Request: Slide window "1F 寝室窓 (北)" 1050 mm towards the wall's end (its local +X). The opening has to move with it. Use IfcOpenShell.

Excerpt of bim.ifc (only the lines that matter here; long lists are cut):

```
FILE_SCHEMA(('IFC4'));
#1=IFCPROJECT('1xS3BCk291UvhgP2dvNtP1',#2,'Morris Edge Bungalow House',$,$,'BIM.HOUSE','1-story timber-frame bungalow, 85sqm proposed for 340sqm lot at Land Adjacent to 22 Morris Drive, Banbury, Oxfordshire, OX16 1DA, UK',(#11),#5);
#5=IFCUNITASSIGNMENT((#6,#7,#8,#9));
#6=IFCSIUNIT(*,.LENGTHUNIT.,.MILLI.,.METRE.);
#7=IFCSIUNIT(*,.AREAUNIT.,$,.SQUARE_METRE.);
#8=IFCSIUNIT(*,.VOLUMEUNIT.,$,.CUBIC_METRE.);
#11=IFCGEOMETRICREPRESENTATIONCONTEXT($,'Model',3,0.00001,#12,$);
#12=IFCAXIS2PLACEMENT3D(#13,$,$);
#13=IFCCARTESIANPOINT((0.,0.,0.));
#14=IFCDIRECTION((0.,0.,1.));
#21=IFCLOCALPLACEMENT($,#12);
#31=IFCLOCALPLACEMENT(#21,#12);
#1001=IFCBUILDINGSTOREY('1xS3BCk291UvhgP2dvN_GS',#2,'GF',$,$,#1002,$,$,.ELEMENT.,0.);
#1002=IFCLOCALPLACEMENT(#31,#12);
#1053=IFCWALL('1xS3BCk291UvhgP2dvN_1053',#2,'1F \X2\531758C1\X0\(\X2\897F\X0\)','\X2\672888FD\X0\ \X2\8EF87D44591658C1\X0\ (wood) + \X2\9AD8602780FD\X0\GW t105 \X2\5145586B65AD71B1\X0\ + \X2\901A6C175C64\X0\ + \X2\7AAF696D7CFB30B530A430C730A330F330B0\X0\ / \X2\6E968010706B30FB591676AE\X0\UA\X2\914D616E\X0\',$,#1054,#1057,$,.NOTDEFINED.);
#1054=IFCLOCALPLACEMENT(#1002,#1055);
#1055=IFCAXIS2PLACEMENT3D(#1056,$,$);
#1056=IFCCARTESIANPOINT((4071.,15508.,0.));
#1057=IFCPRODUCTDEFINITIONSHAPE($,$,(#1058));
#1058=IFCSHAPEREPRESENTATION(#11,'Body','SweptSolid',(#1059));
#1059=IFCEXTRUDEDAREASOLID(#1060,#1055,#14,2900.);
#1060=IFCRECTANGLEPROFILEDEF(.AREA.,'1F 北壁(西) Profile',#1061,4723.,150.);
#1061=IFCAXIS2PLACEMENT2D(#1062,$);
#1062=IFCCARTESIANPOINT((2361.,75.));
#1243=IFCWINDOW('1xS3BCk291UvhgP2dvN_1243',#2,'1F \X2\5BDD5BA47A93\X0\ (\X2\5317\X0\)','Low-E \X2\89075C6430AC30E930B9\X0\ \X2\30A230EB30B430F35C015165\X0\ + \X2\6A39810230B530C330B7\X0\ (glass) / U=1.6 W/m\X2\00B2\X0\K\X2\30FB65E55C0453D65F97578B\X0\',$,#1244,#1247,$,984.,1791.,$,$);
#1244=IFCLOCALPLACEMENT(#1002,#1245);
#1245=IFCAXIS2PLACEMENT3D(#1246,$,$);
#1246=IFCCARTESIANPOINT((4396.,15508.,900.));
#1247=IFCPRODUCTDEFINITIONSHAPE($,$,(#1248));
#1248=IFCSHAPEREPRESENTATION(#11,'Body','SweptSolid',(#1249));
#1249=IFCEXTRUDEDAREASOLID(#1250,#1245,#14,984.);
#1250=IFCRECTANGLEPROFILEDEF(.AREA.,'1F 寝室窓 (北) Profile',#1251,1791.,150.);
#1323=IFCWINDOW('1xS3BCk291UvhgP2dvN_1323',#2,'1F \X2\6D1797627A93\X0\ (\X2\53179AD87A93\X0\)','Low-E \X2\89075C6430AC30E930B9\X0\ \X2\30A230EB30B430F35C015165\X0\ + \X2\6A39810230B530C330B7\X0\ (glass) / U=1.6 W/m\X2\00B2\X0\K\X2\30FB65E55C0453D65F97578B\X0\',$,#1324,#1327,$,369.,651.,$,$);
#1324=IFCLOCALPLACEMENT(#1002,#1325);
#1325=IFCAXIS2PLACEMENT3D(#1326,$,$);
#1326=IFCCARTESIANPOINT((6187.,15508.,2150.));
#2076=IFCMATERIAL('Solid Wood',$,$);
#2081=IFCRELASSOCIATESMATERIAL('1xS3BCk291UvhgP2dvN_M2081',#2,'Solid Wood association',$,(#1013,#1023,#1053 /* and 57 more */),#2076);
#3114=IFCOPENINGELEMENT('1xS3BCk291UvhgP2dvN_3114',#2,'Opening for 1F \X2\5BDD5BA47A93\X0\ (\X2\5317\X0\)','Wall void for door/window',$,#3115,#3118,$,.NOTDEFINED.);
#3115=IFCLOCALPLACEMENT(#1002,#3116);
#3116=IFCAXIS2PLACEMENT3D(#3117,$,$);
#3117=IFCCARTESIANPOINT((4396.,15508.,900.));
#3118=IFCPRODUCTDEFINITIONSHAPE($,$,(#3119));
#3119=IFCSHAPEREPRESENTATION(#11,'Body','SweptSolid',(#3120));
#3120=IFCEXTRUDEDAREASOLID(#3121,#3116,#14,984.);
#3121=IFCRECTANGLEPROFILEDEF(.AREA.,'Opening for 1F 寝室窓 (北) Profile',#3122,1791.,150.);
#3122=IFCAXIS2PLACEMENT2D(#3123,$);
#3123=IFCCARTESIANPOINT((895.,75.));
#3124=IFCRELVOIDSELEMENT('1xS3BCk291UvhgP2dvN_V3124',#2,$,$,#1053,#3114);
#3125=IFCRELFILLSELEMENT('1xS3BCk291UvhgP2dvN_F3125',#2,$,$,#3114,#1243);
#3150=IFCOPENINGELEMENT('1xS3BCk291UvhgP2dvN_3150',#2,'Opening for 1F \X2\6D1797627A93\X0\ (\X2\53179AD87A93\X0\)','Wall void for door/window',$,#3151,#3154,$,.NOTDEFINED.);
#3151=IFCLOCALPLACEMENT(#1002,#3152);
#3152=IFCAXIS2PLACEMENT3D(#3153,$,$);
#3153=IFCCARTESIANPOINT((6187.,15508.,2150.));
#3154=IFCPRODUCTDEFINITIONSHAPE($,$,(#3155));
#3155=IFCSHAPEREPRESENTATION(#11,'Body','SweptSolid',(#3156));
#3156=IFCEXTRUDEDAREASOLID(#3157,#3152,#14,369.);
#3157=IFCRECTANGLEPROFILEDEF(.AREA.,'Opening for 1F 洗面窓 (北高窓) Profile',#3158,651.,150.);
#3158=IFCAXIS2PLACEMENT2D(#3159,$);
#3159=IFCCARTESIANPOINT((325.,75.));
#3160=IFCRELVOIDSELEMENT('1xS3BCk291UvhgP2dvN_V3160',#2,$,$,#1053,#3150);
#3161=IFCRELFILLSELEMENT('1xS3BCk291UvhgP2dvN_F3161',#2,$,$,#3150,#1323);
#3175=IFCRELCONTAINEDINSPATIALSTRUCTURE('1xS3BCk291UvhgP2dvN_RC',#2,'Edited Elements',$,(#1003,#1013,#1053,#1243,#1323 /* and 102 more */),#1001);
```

```python
import ifcopenshell
import ifcopenshell.api.geometry
import ifcopenshell.util.placement

model = ifcopenshell.open("bim.ifc")

window = model.by_id(1243)
opening = window.FillsVoids[0].RelatingOpeningElement
wall = opening.VoidsElements[0].RelatingBuildingElement

wall_matrix = ifcopenshell.util.placement.get_local_placement(wall.ObjectPlacement)
shift = wall_matrix[:3, 0] * 1050.0
before = ifcopenshell.util.placement.get_local_placement(window.ObjectPlacement)[:3, 3].copy()

# The window is not placed relative to its opening, so move both.
for product in (opening, window):
    matrix = ifcopenshell.util.placement.get_local_placement(product.ObjectPlacement)
    matrix[:3, 3] += shift
    ifcopenshell.api.geometry.edit_object_placement(model, product=product, matrix=matrix, is_si=False)

after = ifcopenshell.util.placement.get_local_placement(window.ObjectPlacement)[:3, 3]
print("window moved by", (after - before).round(3) + 0.0)

model.write("bim_rev.ifc")
```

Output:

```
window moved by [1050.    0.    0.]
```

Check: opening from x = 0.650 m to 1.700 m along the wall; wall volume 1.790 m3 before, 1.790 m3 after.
